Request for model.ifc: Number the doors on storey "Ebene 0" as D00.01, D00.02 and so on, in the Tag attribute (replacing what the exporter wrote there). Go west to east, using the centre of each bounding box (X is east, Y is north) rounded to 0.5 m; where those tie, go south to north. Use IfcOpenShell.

First a look at what the model holds.

```python
import ifcopenshell
import ifcopenshell.util.element
import ifcopenshell.util.placement

model = ifcopenshell.open("model.ifc")
print(model.schema)
storey = next(s for s in model.by_type("IfcBuildingStorey") if s.Name == "Ebene 0")
doors = [e for e in ifcopenshell.util.element.get_decomposition(storey) if e.is_a("IfcDoor")]
for e in sorted(doors, key=lambda e: e.id()):
    origin = ifcopenshell.util.placement.get_local_placement(e.ObjectPlacement)[:3, 3]
    print(e.id(), e.Tag, e.Name, origin.round(2) + 0.0, sep=" | ")
```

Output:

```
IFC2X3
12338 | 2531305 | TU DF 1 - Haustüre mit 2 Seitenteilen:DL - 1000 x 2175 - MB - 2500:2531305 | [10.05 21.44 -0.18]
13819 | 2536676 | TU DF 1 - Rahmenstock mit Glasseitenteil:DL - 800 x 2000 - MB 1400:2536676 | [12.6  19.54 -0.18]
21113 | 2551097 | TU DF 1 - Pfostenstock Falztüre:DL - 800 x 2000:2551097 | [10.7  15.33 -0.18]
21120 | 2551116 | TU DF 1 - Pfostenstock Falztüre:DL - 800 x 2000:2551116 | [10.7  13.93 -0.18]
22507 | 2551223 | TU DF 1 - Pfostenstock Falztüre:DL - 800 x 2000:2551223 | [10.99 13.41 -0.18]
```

```python
import ifcopenshell
import ifcopenshell.geom
import ifcopenshell.util.element
import ifcopenshell.util.shape

model = ifcopenshell.open("model.ifc")
settings = ifcopenshell.geom.settings()
settings.set("use-world-coords", True)


def centre(element):
    shape = ifcopenshell.geom.create_shape(settings, element)
    return ifcopenshell.util.shape.get_bbox_centroid(shape.geometry)


storey = next(s for s in model.by_type("IfcBuildingStorey") if s.Name == "Ebene 0")
doors = [e for e in ifcopenshell.util.element.get_decomposition(storey) if e.is_a("IfcDoor")]

# Insertion points can sit at a corner or the storey origin, so sort by the geometry (in metres).
centres = {e: centre(e) for e in doors}
doors.sort(key=lambda e: (round(centres[e][0] / 0.5), centres[e][1]))

for i, e in enumerate(doors, start=1):
    number = f"D00.{i:02d}"
    e.Tag = number
    print(e.id(), number)

model.write("model_rev.ifc")
```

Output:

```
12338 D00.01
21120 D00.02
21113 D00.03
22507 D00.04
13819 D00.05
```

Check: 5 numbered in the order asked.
